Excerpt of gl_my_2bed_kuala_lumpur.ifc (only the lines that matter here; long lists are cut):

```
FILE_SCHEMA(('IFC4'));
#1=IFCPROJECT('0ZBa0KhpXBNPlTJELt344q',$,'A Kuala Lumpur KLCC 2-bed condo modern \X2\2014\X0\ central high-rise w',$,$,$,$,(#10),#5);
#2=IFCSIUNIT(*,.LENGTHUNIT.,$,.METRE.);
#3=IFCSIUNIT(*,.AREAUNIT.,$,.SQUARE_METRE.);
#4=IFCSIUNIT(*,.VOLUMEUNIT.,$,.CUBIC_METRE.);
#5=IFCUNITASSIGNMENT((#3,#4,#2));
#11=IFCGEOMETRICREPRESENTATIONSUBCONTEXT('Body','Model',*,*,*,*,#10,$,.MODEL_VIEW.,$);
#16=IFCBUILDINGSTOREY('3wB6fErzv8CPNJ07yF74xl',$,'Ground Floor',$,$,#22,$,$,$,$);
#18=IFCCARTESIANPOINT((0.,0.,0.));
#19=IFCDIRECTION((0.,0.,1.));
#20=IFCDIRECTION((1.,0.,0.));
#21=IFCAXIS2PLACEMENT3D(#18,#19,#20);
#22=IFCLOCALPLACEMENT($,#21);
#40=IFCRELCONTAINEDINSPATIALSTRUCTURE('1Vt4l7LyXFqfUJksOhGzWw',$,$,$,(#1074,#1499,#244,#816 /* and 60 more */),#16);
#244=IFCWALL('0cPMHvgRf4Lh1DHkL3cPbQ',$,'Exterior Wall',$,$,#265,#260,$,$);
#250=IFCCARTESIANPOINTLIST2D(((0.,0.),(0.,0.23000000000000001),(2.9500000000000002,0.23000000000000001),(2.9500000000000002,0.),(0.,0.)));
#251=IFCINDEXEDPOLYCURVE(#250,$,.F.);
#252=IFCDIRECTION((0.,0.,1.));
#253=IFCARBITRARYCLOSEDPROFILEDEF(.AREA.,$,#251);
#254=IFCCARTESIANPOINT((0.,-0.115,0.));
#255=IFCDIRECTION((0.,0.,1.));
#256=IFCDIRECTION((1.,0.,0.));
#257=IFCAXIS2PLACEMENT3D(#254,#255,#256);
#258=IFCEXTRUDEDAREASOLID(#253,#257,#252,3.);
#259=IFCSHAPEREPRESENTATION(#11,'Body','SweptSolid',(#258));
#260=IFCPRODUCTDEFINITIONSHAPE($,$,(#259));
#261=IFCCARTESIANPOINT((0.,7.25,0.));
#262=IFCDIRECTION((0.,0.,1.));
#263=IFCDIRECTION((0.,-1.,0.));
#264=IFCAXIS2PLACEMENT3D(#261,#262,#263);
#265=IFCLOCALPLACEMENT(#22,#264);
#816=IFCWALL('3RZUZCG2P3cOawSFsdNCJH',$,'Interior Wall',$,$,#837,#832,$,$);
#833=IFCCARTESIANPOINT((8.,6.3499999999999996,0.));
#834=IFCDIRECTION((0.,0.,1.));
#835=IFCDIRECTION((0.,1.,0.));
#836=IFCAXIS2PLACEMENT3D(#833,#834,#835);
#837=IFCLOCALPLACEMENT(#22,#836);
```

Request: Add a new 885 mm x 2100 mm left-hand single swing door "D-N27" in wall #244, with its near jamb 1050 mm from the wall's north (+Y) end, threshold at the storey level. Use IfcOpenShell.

```python
import numpy as np
import ifcopenshell
import ifcopenshell.api.feature
import ifcopenshell.api.geometry
import ifcopenshell.api.root
import ifcopenshell.api.spatial
import ifcopenshell.geom
import ifcopenshell.util.element
import ifcopenshell.util.placement
import ifcopenshell.util.representation
import ifcopenshell.util.shape
import ifcopenshell.util.unit

model = ifcopenshell.open("gl_my_2bed_kuala_lumpur.ifc")
unit_scale = ifcopenshell.util.unit.calculate_unit_scale(model)
settings = ifcopenshell.geom.settings()


def volume(element):
    """Net volume in cubic metres, openings subtracted."""
    shape = ifcopenshell.geom.create_shape(settings, element)
    return ifcopenshell.util.shape.get_volume(shape.geometry)


wall = model.by_guid("0cPMHvgRf4Lh1DHkL3cPbQ")
storey = ifcopenshell.util.element.get_container(wall, ifc_class="IfcBuildingStorey")
context = ifcopenshell.util.representation.get_context(model, "Model", "Body", "MODEL_VIEW")
before = volume(wall)

width, height, from_end, sill = 0.885, 2.1, 1.05, 0.0  # metres

# The wall runs along its own X axis, and the end named is its -X end.
wall_shape = ifcopenshell.geom.create_shape(settings, wall)
x, y, z = ifcopenshell.util.shape.get_vertices(wall_shape.geometry).T
start = x.min() + from_end
face, thickness = float(y.min()), float(y.max() - y.min())
wall_matrix = ifcopenshell.util.placement.get_local_placement(wall.ObjectPlacement)
level = ifcopenshell.util.placement.get_local_placement(storey.ObjectPlacement)[2, 3]


def in_wall(x, y):
    """Placement at x, y metres in the wall's axes, at sill height."""
    matrix = wall_matrix.copy()
    matrix[:, 3] = wall_matrix @ np.array([x / unit_scale, y / unit_scale, 0.0, 1.0])
    matrix[2, 3] = level + sill / unit_scale
    return matrix


# Opening: a box that overshoots both wall faces by 50 mm.
opening = ifcopenshell.api.root.create_entity(model, ifc_class="IfcOpeningElement", predefined_type="OPENING")
box = ifcopenshell.api.geometry.add_wall_representation(
    model, context=context, length=width, height=height, thickness=thickness + 0.1
)
ifcopenshell.api.geometry.assign_representation(model, product=opening, representation=box)
ifcopenshell.api.geometry.edit_object_placement(model, product=opening, matrix=in_wall(start, face - 0.05), is_si=False)
ifcopenshell.api.feature.add_feature(model, feature=opening, element=wall)

door = ifcopenshell.api.root.create_entity(model, ifc_class="IfcDoor", name="D-N27", predefined_type="DOOR")
door.OverallWidth, door.OverallHeight = width / unit_scale, height / unit_scale
door.OperationType = "SINGLE_SWING_LEFT"
body = ifcopenshell.api.geometry.add_door_representation(
    model,
    context=context,
    overall_width=door.OverallWidth,
    overall_height=door.OverallHeight,
    operation_type="SINGLE_SWING_LEFT",
    lining_properties={"LiningDepth": thickness / unit_scale, "ThresholdDepth": thickness / unit_scale},
)
ifcopenshell.api.geometry.assign_representation(model, product=door, representation=body)
ifcopenshell.api.spatial.assign_container(model, products=[door], relating_structure=storey)
ifcopenshell.api.feature.add_filling(model, opening=opening, element=door)

# The lining spans the wall, so the door starts at the wall face.
ifcopenshell.api.geometry.edit_object_placement(model, product=door, matrix=in_wall(start, face), is_si=False)

after = volume(wall)

print(f"wall volume {before:.3f} -> {after:.3f} m3")

model.write("gl_my_2bed_kuala_lumpur_rev.ifc")
```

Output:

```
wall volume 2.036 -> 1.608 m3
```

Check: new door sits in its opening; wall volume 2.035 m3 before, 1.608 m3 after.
